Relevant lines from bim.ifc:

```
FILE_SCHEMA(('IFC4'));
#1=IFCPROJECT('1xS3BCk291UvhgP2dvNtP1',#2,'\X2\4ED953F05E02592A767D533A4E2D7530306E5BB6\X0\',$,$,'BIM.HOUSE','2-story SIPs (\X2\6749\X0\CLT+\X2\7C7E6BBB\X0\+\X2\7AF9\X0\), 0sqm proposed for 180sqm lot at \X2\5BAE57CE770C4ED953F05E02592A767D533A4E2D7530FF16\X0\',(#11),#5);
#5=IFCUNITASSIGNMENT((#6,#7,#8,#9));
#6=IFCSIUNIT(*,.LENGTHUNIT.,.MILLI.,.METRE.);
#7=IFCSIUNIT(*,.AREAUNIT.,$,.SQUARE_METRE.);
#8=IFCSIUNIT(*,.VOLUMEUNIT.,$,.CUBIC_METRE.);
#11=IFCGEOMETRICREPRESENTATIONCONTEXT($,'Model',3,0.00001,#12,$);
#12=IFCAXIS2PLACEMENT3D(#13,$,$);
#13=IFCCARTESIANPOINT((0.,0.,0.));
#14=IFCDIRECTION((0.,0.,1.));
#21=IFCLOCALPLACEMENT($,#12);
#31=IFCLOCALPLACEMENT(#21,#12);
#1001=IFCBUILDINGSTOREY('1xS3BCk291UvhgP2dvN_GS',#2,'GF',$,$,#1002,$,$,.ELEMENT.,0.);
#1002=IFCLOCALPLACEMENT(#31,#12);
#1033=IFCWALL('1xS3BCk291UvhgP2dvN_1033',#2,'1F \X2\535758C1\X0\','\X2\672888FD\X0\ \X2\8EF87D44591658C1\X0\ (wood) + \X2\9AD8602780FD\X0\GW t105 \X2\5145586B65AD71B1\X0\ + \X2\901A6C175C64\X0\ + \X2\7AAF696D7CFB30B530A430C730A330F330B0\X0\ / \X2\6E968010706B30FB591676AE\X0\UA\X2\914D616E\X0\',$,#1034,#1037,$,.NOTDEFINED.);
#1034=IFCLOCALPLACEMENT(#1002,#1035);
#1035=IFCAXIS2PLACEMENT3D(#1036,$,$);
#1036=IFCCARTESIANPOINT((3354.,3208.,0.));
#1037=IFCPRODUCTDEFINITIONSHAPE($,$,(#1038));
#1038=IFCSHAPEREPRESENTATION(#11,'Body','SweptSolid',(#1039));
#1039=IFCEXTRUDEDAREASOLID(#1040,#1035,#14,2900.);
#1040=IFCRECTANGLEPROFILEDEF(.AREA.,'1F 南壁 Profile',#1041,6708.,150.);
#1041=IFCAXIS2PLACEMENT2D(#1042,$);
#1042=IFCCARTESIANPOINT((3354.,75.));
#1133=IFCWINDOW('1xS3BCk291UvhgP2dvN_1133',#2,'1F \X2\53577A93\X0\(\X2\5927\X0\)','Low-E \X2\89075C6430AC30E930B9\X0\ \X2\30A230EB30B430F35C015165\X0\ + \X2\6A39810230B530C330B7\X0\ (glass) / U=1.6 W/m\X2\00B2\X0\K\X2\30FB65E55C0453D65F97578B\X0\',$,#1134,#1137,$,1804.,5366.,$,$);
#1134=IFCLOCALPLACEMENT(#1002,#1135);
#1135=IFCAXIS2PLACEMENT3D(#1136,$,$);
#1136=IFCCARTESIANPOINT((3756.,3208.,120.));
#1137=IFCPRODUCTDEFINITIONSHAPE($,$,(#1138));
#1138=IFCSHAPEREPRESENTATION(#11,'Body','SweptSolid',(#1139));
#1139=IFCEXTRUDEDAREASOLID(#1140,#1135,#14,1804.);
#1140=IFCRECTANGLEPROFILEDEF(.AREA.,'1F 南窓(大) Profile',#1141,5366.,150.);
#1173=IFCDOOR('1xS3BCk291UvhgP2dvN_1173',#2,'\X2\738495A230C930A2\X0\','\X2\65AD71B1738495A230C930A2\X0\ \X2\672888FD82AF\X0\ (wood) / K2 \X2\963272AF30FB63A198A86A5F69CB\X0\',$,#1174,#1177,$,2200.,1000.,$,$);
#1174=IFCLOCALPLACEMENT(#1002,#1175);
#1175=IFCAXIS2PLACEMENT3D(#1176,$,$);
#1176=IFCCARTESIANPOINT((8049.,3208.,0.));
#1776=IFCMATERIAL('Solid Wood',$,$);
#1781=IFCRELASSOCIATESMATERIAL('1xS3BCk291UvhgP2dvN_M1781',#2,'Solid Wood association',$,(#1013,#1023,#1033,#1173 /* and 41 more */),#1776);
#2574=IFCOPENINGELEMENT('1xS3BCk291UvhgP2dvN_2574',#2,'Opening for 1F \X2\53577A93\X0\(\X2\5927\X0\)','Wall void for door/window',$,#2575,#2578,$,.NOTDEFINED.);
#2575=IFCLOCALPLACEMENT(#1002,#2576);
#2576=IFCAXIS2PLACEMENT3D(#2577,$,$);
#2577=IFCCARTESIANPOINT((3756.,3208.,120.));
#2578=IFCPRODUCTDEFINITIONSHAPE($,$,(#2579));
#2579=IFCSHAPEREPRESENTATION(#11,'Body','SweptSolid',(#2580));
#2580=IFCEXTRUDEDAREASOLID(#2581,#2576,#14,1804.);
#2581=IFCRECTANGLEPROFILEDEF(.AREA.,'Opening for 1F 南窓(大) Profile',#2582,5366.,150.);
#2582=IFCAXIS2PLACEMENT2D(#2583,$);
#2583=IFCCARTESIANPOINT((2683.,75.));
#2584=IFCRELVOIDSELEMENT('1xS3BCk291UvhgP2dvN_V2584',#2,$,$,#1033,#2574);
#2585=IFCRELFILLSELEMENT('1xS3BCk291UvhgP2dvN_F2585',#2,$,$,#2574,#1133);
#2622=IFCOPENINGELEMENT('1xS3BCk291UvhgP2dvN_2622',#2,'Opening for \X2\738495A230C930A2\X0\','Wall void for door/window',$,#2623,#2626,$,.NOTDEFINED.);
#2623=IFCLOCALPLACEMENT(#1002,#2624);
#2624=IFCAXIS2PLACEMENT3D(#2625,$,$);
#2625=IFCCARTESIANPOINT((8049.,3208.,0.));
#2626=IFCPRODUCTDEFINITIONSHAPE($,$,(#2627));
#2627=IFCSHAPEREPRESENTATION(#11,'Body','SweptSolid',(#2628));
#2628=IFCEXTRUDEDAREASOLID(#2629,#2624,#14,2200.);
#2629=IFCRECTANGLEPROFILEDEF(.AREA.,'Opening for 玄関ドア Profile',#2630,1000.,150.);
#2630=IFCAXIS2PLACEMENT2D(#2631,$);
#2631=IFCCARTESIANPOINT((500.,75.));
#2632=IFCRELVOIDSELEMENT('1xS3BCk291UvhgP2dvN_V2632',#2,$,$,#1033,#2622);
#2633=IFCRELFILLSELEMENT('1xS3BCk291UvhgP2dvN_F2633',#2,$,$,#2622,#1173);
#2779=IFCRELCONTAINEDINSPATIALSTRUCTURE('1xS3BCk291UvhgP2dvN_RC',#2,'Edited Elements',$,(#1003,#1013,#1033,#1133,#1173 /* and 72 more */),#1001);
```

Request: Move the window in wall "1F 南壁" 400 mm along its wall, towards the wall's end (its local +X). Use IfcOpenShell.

```python
import ifcopenshell
import ifcopenshell.api.geometry
import ifcopenshell.util.placement

model = ifcopenshell.open("bim.ifc")

window = model.by_guid("1xS3BCk291UvhgP2dvN_1133")
opening = window.FillsVoids[0].RelatingOpeningElement
wall = opening.VoidsElements[0].RelatingBuildingElement

wall_matrix = ifcopenshell.util.placement.get_local_placement(wall.ObjectPlacement)
shift = wall_matrix[:3, 0] * 400.0
before = ifcopenshell.util.placement.get_local_placement(window.ObjectPlacement)[:3, 3].copy()

# The window is not placed relative to its opening, so move both.
for product in (opening, window):
    matrix = ifcopenshell.util.placement.get_local_placement(product.ObjectPlacement)
    matrix[:3, 3] += shift
    ifcopenshell.api.geometry.edit_object_placement(model, product=product, matrix=matrix, is_si=False)

after = ifcopenshell.util.placement.get_local_placement(window.ObjectPlacement)[:3, 3]
print("window moved by", (after - before).round(3) + 0.0)

model.write("bim_edited.ifc")
```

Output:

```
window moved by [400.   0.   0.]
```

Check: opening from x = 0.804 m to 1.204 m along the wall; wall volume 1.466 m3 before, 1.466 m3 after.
